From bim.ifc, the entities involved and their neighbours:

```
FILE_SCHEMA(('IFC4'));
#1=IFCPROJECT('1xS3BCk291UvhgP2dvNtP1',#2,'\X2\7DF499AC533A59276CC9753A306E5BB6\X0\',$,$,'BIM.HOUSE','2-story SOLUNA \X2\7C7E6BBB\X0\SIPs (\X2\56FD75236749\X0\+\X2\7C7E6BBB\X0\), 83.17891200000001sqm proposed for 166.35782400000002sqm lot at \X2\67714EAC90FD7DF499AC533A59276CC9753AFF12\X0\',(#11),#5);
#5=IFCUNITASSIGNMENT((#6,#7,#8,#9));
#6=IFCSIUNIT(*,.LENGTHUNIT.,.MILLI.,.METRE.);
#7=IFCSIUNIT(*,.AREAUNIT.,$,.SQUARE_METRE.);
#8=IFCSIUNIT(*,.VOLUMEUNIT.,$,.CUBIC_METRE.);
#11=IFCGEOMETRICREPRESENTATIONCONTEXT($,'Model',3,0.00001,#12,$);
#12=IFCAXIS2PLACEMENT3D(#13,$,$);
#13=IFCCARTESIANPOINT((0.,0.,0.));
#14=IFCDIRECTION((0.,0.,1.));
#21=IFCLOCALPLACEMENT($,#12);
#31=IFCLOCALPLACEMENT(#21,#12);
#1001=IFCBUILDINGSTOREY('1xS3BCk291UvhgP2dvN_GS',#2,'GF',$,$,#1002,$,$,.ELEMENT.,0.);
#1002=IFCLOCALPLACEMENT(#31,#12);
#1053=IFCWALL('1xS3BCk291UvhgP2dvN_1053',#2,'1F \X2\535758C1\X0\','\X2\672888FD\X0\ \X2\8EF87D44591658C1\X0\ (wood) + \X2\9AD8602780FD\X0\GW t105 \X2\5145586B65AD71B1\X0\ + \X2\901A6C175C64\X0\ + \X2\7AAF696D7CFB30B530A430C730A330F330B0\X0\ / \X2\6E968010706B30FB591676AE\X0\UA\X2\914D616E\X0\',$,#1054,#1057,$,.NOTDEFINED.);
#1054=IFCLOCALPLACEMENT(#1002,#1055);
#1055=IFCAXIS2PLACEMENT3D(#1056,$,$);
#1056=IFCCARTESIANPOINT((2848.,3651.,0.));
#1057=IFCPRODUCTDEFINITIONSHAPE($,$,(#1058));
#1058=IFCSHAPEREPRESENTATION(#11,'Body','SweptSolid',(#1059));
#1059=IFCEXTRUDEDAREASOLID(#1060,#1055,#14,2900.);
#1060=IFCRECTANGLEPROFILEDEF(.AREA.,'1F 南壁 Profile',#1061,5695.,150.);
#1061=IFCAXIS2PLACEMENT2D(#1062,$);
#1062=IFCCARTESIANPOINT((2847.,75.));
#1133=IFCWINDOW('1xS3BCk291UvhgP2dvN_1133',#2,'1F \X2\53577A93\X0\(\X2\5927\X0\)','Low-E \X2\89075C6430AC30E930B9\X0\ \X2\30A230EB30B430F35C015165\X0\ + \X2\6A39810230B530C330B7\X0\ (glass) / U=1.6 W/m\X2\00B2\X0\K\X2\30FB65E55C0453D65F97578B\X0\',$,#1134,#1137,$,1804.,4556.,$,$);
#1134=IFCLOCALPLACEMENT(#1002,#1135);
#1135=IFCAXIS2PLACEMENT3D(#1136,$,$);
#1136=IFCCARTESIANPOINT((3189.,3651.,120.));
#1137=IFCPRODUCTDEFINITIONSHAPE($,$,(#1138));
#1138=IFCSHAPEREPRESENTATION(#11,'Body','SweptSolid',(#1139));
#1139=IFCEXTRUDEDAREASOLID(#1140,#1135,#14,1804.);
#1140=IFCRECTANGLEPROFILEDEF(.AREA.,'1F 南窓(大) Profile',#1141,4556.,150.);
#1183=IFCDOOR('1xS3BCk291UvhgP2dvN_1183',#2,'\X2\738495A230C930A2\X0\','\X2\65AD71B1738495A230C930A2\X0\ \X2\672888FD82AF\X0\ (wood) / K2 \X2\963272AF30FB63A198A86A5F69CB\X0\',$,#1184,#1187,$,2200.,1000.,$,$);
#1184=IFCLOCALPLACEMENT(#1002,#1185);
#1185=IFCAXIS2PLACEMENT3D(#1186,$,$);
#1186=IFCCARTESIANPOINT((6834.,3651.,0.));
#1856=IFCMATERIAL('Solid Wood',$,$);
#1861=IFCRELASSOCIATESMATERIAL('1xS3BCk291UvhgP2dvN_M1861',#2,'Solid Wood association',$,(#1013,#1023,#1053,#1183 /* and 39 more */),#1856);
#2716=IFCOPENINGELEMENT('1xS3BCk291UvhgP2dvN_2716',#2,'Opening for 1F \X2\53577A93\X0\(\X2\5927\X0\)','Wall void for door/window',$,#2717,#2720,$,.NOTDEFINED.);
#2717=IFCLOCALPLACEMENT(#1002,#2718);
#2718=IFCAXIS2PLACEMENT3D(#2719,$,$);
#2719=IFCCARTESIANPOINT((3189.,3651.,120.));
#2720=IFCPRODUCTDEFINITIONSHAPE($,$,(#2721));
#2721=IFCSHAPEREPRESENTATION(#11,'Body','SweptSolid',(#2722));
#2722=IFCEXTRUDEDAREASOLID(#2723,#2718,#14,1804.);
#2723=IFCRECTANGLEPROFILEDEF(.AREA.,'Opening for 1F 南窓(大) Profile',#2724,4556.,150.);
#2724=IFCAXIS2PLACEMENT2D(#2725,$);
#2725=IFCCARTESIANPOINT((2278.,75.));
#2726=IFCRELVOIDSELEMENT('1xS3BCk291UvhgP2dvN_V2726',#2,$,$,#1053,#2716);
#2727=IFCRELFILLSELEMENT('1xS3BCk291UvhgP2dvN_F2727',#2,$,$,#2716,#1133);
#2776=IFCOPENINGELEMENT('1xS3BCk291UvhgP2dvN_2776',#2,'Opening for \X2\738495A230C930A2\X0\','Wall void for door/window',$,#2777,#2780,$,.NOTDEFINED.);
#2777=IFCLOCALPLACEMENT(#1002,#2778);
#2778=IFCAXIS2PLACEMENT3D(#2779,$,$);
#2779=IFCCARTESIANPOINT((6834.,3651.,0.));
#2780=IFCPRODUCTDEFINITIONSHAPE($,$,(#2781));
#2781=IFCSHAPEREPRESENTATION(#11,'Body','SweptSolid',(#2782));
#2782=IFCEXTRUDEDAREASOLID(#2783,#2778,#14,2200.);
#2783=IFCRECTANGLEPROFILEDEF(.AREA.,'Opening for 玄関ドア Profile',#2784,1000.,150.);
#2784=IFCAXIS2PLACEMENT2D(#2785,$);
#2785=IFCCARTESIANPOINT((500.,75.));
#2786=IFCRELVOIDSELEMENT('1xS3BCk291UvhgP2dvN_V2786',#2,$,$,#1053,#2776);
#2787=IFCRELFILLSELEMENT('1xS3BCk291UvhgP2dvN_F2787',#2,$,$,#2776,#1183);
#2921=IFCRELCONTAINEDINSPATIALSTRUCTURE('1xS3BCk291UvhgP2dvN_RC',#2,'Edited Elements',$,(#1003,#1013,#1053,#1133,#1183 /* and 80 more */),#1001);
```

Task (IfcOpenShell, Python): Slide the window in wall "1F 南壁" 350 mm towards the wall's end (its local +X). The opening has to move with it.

```python
import ifcopenshell
import ifcopenshell.api.geometry
import ifcopenshell.util.placement

model = ifcopenshell.open("bim.ifc")

window = model.by_id(1133)
opening = window.FillsVoids[0].RelatingOpeningElement
wall = opening.VoidsElements[0].RelatingBuildingElement

wall_matrix = ifcopenshell.util.placement.get_local_placement(wall.ObjectPlacement)
shift = wall_matrix[:3, 0] * 350.0
before = ifcopenshell.util.placement.get_local_placement(window.ObjectPlacement)[:3, 3].copy()

# The window is not placed relative to its opening, so move both.
for product in (opening, window):
    matrix = ifcopenshell.util.placement.get_local_placement(product.ObjectPlacement)
    matrix[:3, 3] += shift
    ifcopenshell.api.geometry.edit_object_placement(model, product=product, matrix=matrix, is_si=False)

after = ifcopenshell.util.placement.get_local_placement(window.ObjectPlacement)[:3, 3]
print("window moved by", (after - before).round(3) + 0.0)

model.write("bim_rev.ifc")
```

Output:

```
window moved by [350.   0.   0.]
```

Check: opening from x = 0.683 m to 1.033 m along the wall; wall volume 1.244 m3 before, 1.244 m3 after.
